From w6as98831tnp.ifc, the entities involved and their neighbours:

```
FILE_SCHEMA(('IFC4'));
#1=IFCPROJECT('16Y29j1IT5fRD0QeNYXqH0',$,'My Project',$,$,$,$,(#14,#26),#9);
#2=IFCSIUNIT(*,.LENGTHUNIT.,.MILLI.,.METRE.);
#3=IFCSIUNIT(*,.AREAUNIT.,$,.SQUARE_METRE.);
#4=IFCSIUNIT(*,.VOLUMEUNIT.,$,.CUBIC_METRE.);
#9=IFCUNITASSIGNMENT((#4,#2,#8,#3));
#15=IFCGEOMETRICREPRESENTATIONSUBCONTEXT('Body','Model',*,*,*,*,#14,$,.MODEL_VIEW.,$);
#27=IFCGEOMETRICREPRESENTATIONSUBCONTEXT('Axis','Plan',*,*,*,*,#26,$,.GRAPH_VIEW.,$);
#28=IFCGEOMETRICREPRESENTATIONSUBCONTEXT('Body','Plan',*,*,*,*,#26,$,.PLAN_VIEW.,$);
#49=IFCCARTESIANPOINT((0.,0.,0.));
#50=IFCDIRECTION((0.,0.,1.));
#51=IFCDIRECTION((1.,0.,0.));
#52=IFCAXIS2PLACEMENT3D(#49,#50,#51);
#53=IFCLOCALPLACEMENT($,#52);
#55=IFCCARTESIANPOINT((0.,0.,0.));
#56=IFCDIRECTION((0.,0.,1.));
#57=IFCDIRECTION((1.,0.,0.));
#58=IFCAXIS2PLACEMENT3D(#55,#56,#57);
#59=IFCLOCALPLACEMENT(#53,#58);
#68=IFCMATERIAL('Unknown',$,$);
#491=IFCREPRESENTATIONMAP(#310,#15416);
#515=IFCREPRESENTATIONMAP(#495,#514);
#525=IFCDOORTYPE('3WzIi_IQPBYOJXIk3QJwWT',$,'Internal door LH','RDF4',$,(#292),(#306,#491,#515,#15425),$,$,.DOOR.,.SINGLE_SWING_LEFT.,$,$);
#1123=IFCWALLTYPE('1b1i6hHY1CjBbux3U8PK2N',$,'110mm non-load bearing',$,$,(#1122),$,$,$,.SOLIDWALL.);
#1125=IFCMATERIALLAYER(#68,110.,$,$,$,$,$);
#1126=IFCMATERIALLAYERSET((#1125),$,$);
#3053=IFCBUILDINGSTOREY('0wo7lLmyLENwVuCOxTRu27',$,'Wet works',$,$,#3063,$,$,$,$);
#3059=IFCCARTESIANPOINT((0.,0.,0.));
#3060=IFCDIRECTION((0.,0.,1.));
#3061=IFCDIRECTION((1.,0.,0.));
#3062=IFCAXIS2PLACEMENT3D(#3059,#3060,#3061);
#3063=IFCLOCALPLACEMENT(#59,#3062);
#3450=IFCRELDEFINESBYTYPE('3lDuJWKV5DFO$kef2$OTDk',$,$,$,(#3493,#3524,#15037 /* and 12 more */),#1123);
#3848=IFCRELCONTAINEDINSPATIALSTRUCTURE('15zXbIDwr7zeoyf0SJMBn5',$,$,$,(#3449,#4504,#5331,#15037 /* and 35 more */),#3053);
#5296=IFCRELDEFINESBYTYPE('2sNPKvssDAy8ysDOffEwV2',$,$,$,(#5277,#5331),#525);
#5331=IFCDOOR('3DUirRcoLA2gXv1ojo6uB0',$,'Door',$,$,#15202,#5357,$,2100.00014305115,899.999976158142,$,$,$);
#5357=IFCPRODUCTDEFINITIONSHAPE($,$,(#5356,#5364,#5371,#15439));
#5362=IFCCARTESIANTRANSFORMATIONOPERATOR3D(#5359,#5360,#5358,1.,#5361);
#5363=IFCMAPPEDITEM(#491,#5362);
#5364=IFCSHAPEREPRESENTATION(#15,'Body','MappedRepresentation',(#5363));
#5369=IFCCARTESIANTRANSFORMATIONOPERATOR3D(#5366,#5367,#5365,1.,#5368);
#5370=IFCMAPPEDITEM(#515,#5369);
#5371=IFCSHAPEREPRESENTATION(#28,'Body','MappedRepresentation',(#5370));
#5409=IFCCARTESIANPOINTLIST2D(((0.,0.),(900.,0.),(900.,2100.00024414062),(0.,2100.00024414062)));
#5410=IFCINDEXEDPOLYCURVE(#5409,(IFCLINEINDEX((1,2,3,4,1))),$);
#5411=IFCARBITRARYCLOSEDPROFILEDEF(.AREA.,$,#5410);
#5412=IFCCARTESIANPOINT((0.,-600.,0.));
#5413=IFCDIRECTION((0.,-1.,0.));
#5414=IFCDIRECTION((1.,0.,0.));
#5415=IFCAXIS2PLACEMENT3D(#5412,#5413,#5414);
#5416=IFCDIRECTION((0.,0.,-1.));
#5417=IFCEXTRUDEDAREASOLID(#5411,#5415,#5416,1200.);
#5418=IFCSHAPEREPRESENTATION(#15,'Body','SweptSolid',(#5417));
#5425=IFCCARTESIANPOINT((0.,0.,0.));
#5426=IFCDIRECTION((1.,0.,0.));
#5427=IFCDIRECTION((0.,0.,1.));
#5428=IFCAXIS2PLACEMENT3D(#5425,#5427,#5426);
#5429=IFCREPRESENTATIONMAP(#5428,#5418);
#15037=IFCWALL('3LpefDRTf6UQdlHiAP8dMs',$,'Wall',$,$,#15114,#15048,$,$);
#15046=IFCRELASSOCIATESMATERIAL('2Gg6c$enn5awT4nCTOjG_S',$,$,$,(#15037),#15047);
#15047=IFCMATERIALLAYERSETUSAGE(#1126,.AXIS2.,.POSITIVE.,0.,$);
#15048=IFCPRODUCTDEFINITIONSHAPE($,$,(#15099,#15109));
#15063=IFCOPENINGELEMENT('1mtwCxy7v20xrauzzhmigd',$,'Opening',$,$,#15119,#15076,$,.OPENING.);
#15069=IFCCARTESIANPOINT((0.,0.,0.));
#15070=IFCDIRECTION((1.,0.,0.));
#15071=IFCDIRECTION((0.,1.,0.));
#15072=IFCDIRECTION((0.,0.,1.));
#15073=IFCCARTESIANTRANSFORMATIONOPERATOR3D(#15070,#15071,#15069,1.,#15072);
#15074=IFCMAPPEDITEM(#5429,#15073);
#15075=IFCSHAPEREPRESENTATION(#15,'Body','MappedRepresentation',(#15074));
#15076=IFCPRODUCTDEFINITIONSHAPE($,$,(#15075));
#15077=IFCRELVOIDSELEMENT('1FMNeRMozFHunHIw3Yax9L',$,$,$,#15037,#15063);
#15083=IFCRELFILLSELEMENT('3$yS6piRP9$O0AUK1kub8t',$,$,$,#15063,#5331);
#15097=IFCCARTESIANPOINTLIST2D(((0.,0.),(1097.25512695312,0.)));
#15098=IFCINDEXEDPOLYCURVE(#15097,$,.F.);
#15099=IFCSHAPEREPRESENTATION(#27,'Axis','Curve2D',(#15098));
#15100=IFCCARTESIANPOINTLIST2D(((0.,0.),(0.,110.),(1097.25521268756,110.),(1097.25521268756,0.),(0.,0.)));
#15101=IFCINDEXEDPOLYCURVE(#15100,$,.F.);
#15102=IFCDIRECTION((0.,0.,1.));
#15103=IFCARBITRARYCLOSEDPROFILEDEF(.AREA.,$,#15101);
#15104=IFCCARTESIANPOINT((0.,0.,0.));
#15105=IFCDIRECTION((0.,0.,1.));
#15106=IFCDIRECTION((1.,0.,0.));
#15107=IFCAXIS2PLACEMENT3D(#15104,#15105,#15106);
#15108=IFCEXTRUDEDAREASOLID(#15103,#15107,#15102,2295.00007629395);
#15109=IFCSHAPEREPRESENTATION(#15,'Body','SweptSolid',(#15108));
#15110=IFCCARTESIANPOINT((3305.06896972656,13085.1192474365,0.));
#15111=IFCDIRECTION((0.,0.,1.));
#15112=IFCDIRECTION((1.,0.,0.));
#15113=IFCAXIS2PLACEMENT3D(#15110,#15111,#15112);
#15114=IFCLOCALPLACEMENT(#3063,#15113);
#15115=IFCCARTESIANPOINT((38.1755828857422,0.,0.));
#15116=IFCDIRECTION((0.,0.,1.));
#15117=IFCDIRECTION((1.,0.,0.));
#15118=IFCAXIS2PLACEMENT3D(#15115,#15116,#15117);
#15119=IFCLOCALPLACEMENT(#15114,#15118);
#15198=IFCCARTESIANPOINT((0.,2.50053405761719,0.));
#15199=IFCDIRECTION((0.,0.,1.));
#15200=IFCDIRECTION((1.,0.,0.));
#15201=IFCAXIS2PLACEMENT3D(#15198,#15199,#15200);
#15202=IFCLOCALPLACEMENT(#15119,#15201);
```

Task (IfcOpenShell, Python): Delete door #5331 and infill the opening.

```python
import ifcopenshell
import ifcopenshell.api.feature
import ifcopenshell.api.root
import ifcopenshell.geom
import ifcopenshell.util.shape

model = ifcopenshell.open("w6as98831tnp.ifc")
settings = ifcopenshell.geom.settings()


def volume(element):
    """Net volume in cubic metres, openings subtracted."""
    shape = ifcopenshell.geom.create_shape(settings, element)
    return ifcopenshell.util.shape.get_volume(shape.geometry)


door = model.by_id(5331)
opening = door.FillsVoids[0].RelatingOpeningElement
wall = opening.VoidsElements[0].RelatingBuildingElement
before = volume(wall)

ifcopenshell.api.root.remove_product(model, product=door)
ifcopenshell.api.feature.remove_feature(model, feature=opening)

after = volume(wall)

print(f"wall volume {before:.3f} -> {after:.3f} m3")

model.write("w6as98831tnp_edited.ifc")
```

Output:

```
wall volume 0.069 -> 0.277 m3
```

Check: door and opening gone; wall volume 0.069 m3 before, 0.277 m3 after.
